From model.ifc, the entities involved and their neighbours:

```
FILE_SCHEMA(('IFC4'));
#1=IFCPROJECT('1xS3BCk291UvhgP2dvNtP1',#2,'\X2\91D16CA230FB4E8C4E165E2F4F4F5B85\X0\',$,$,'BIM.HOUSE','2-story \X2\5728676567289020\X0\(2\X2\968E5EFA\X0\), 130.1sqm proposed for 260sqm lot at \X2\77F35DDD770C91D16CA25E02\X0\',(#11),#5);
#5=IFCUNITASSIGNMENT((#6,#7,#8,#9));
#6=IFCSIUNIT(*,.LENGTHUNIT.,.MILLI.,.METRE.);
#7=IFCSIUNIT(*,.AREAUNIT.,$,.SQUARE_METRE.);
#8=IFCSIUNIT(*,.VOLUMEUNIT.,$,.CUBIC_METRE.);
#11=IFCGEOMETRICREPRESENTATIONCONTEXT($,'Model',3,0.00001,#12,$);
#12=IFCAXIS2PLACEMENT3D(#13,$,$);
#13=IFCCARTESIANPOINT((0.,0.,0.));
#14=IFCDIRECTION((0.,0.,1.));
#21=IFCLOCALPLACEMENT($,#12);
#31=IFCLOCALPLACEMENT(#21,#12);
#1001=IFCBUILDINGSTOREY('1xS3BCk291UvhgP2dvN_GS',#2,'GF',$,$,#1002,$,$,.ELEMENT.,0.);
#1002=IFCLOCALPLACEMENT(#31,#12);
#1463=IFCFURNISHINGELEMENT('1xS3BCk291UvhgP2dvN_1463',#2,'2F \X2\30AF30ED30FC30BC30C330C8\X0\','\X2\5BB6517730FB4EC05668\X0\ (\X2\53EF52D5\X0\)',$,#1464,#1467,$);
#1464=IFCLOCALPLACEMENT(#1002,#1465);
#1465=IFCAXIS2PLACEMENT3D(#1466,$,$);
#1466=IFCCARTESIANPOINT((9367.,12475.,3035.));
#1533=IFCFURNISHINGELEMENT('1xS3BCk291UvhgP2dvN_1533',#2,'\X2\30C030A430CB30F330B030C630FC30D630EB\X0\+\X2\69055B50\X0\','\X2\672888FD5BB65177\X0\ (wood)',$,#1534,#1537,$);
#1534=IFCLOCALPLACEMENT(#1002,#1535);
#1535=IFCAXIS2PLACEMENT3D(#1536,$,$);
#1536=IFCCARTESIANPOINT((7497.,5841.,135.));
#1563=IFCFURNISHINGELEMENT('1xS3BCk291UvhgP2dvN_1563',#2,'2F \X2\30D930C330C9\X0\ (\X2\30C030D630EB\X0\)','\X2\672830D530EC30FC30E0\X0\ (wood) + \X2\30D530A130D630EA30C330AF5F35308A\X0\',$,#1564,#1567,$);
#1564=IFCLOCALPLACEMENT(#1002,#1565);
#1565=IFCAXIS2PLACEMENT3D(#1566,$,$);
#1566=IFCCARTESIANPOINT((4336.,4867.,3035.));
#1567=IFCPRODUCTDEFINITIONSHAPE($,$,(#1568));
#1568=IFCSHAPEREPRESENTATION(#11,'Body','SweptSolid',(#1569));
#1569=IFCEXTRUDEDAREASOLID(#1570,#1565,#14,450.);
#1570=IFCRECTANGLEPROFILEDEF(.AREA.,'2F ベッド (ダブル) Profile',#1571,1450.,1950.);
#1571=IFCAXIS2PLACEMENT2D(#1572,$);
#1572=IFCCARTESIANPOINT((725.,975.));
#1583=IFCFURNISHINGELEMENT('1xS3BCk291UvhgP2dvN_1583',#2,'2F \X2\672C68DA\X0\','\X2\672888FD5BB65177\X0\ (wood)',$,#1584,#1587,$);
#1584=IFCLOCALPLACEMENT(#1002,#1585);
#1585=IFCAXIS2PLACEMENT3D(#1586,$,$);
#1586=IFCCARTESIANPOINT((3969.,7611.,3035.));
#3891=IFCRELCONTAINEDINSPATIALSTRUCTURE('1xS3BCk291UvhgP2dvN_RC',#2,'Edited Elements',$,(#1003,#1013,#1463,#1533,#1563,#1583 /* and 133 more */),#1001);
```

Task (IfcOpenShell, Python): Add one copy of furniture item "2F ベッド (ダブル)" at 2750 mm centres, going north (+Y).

```python
import numpy as np
import ifcopenshell
import ifcopenshell.api.geometry
import ifcopenshell.api.root
import ifcopenshell.util.element
import ifcopenshell.util.placement

model = ifcopenshell.open("model.ifc")


def reuse_history(source, copy):
    """copy_class also copies each property set's owner history, people and application; keep the originals."""
    for rel in copy.IsDefinedBy:
        if rel.is_a("IfcRelDefinesByProperties") and (history := rel.RelatingPropertyDefinition.OwnerHistory):
            rel.RelatingPropertyDefinition.OwnerHistory = source.OwnerHistory
            ifcopenshell.util.element.remove_deep2(model, history)


source = model.by_guid("1xS3BCk291UvhgP2dvN_1563")
base = ifcopenshell.util.placement.get_local_placement(source.ObjectPlacement)
step = np.array([0.0, 1.0, 0.0]) * 2750.0

for i in range(1, 2):
    copy = ifcopenshell.api.root.copy_class(model, product=source)
    copy.Representation = ifcopenshell.util.element.copy_deep(
        model, source.Representation, exclude=["IfcGeometricRepresentationContext", "IfcRepresentationMap"]
    )
    reuse_history(source, copy)
    matrix = base.copy()
    matrix[:3, 3] += i * step
    print("added at", matrix[:3, 3].round(3) + 0.0)
    ifcopenshell.api.geometry.edit_object_placement(model, product=copy, matrix=matrix, is_si=False)

model.write("model_v2.ifc")
```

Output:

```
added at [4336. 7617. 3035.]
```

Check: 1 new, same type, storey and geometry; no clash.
